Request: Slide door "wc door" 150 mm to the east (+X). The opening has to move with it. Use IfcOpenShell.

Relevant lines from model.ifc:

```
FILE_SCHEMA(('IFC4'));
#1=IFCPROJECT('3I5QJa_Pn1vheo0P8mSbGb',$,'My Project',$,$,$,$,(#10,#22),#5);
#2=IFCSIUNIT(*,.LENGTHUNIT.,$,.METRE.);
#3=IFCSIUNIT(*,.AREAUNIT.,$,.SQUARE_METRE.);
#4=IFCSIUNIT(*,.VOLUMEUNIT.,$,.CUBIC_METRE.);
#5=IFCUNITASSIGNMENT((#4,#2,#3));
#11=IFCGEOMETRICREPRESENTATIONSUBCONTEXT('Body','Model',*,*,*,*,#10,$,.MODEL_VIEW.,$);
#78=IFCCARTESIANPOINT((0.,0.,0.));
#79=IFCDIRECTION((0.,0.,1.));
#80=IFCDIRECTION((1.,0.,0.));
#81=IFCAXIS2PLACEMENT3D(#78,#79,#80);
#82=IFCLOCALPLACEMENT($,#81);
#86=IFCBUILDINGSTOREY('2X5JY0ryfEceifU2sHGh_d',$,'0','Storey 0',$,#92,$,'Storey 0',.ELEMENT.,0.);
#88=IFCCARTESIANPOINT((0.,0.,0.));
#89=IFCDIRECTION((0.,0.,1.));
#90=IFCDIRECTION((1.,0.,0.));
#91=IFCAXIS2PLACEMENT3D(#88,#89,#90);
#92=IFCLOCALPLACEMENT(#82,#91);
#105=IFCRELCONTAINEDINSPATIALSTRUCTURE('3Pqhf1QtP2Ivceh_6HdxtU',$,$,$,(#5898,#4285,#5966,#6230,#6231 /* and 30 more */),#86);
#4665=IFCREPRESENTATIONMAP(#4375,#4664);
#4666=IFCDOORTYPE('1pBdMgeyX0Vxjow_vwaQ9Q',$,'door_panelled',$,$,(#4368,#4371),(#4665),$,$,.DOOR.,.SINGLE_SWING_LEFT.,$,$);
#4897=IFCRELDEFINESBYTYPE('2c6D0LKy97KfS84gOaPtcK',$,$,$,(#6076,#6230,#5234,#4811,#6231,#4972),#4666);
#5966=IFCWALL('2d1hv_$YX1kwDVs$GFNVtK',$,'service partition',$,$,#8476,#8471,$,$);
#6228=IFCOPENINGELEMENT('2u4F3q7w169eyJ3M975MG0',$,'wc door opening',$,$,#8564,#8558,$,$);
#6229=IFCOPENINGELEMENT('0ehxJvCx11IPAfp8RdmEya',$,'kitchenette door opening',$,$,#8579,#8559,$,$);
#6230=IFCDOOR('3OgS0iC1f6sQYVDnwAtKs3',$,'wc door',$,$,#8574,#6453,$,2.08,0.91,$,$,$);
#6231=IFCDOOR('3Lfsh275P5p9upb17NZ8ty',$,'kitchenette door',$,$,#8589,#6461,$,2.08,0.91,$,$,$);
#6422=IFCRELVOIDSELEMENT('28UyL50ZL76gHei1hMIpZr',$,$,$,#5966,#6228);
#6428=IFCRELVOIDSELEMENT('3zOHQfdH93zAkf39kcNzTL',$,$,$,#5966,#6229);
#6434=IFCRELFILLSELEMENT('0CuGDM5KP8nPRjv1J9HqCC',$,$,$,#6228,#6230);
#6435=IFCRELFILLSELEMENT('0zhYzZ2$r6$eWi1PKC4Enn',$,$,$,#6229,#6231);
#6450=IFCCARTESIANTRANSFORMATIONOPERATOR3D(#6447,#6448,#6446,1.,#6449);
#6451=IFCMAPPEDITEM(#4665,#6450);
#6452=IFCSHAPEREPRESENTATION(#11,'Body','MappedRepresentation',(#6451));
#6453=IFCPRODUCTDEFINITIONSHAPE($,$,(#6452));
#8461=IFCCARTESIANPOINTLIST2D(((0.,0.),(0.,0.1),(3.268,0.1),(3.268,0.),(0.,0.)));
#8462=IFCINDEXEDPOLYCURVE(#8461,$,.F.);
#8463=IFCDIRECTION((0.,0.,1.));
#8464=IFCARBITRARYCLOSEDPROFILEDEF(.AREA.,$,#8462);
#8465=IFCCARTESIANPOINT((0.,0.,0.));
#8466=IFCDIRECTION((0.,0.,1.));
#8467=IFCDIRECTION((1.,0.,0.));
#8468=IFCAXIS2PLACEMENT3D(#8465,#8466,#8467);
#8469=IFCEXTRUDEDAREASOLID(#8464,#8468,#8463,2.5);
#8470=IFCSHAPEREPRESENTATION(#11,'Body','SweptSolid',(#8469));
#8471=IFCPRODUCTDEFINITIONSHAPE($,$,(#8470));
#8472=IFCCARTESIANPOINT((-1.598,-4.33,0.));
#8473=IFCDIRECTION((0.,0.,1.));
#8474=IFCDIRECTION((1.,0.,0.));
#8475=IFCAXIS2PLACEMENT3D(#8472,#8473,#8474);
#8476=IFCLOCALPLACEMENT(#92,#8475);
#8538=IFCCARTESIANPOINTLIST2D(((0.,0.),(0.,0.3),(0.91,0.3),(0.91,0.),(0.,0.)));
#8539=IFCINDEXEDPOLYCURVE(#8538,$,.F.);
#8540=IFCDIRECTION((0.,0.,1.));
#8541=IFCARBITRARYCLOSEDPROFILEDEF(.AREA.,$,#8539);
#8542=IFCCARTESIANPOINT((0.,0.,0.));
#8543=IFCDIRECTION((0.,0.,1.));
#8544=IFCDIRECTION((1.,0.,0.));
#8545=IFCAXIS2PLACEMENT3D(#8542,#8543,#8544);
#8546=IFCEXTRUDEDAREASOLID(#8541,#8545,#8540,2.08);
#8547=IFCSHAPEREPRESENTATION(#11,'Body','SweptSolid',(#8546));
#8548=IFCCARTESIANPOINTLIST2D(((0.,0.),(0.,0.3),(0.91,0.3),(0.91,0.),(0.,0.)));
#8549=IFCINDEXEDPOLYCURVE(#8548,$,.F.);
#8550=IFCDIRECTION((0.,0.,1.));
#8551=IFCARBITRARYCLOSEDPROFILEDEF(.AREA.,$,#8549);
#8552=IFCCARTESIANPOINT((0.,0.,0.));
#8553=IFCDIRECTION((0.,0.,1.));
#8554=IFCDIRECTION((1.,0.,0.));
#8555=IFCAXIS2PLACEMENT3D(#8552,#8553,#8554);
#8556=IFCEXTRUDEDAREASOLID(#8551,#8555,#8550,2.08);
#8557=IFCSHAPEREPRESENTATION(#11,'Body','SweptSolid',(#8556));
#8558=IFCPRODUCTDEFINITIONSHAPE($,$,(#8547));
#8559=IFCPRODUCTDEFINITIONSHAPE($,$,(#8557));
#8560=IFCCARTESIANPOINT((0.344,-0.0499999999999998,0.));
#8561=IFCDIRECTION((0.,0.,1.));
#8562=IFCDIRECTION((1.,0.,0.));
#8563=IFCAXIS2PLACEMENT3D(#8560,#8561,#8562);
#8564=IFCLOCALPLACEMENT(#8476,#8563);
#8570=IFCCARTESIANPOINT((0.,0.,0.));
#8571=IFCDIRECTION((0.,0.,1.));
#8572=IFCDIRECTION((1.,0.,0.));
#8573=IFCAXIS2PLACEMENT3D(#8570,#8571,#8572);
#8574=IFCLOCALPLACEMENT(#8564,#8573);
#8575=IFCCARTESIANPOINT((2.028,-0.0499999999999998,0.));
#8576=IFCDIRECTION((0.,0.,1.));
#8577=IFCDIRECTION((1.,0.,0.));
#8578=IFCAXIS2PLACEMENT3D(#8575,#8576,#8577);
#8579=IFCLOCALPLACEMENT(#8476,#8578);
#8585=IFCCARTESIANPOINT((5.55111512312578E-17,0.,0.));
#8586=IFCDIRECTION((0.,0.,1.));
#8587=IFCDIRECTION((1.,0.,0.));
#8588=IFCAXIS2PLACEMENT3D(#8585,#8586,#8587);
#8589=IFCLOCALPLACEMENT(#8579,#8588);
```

```python
import ifcopenshell
import ifcopenshell.api.geometry
import ifcopenshell.util.placement
import ifcopenshell.util.unit

model = ifcopenshell.open("model.ifc")
unit_scale = ifcopenshell.util.unit.calculate_unit_scale(model)

door = model.by_guid("3OgS0iC1f6sQYVDnwAtKs3")
opening = door.FillsVoids[0].RelatingOpeningElement
wall = opening.VoidsElements[0].RelatingBuildingElement

wall_matrix = ifcopenshell.util.placement.get_local_placement(wall.ObjectPlacement)
shift = wall_matrix[:3, 0] * 0.15 / unit_scale
before = ifcopenshell.util.placement.get_local_placement(door.ObjectPlacement)[:3, 3].copy()

# The door is placed relative to its opening, so it follows when the opening moves.
matrix = ifcopenshell.util.placement.get_local_placement(opening.ObjectPlacement)
matrix[:3, 3] += shift
ifcopenshell.api.geometry.edit_object_placement(
    model, product=opening, matrix=matrix, is_si=False, should_transform_children=True
)

after = ifcopenshell.util.placement.get_local_placement(door.ObjectPlacement)[:3, 3]
print("door moved by", (after - before).round(3) + 0.0)

model.write("model_edited.ifc")
```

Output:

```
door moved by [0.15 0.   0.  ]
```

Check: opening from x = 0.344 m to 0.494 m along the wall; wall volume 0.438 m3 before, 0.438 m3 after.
